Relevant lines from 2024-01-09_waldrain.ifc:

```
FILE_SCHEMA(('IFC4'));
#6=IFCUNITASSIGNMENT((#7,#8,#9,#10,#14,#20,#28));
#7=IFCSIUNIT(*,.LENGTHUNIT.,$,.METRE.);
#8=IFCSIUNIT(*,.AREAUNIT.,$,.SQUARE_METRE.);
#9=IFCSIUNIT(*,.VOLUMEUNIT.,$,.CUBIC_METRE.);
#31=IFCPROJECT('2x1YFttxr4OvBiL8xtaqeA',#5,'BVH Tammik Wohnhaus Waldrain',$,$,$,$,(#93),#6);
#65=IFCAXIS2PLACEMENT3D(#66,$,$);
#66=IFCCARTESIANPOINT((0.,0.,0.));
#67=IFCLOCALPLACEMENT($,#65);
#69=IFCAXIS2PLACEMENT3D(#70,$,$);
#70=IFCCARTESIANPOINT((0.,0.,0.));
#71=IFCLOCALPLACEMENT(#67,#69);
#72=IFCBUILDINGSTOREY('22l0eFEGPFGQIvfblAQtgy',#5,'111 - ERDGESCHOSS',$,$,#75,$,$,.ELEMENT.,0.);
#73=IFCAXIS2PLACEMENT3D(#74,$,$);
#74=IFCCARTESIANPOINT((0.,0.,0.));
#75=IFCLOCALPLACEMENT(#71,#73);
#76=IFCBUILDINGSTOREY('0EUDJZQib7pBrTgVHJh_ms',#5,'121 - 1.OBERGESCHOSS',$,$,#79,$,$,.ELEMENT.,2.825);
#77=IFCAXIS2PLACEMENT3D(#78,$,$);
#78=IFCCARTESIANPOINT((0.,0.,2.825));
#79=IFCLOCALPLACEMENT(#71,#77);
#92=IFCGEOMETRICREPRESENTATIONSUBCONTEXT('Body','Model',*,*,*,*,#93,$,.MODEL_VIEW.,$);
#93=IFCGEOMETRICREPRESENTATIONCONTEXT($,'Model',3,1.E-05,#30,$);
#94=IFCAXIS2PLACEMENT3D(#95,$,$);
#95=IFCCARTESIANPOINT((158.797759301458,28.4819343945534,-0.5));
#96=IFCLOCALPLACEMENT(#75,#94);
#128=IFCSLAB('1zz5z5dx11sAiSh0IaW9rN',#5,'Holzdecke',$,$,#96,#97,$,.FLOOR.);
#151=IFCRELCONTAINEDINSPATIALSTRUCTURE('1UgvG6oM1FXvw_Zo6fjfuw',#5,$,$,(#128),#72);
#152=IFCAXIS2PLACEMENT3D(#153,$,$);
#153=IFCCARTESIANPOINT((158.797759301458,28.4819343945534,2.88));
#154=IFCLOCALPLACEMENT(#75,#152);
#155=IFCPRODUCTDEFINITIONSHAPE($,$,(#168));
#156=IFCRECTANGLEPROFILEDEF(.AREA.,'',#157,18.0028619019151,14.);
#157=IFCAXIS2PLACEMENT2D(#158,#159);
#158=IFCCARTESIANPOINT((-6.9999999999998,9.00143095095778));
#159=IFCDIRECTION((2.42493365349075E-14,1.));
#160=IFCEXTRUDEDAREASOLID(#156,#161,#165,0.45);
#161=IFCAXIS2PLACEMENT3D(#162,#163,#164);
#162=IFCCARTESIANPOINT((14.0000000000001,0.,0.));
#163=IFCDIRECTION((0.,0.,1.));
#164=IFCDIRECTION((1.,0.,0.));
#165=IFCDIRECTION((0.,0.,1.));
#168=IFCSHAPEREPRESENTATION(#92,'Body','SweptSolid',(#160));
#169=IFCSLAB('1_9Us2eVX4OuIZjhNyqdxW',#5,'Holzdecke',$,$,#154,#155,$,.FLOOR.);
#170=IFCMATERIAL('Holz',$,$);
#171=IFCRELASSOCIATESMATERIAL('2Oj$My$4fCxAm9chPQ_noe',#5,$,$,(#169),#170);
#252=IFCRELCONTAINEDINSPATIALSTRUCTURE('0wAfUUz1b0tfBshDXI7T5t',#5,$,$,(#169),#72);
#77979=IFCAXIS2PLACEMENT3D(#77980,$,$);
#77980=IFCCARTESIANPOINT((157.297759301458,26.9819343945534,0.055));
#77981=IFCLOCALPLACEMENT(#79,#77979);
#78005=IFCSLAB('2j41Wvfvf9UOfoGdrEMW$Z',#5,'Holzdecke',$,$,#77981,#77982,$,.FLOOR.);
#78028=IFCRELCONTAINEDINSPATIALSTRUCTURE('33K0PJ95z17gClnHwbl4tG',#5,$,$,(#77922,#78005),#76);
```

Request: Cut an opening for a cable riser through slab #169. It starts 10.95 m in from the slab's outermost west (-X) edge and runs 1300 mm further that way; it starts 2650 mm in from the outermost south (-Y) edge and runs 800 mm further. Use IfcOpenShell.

```python
import numpy as np
import ifcopenshell
import ifcopenshell.api.feature
import ifcopenshell.api.geometry
import ifcopenshell.api.root
import ifcopenshell.geom
import ifcopenshell.util.placement
import ifcopenshell.util.representation
import ifcopenshell.util.shape
import ifcopenshell.util.unit

model = ifcopenshell.open("2024-01-09_waldrain.ifc")
unit_scale = ifcopenshell.util.unit.calculate_unit_scale(model)
settings = ifcopenshell.geom.settings()


def volume(element):
    """Net volume in cubic metres, openings subtracted."""
    shape = ifcopenshell.geom.create_shape(settings, element)
    return ifcopenshell.util.shape.get_volume(shape.geometry)


slab = model.by_id(169)
before = volume(slab)

# Extent in the slab's own axes, in metres. The edges named are its -X and -Y sides.
slab_shape = ifcopenshell.geom.create_shape(settings, slab)
vertices = ifcopenshell.util.shape.get_vertices(slab_shape.geometry)
x_min, y_min, bottom = vertices.min(axis=0)
top = vertices[:, 2].max()

opening = ifcopenshell.api.root.create_entity(model, ifc_class="IfcOpeningElement", name="Cable riser opening", predefined_type="OPENING")
context = ifcopenshell.util.representation.get_context(model, "Model", "Body", "MODEL_VIEW")
width, depth = 1.3, 0.8
outline = [(0.0, 0.0), (width, 0.0), (width, depth), (0.0, depth), (0.0, 0.0)]
# Overshoot both faces by 50 mm so the cut is clean.
shape = ifcopenshell.api.geometry.add_slab_representation(
    model, context=context, depth=top - bottom + 0.1, polyline=outline
)
ifcopenshell.api.geometry.assign_representation(model, product=opening, representation=shape)

matrix = ifcopenshell.util.placement.get_local_placement(slab.ObjectPlacement)
matrix[:, 3] = matrix @ np.append(np.array([x_min + 10.95, y_min + 2.65, bottom - 0.05]) / unit_scale, 1.0)
ifcopenshell.api.geometry.edit_object_placement(model, product=opening, matrix=matrix, is_si=False)
ifcopenshell.api.feature.add_feature(model, feature=opening, element=slab)

after = volume(slab)

print(f"slab volume {before:.3f} -> {after:.3f} m3")

model.write("2024-01-09_waldrain_updated.ifc")
```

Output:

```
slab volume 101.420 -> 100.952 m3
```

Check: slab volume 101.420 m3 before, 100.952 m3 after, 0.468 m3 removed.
